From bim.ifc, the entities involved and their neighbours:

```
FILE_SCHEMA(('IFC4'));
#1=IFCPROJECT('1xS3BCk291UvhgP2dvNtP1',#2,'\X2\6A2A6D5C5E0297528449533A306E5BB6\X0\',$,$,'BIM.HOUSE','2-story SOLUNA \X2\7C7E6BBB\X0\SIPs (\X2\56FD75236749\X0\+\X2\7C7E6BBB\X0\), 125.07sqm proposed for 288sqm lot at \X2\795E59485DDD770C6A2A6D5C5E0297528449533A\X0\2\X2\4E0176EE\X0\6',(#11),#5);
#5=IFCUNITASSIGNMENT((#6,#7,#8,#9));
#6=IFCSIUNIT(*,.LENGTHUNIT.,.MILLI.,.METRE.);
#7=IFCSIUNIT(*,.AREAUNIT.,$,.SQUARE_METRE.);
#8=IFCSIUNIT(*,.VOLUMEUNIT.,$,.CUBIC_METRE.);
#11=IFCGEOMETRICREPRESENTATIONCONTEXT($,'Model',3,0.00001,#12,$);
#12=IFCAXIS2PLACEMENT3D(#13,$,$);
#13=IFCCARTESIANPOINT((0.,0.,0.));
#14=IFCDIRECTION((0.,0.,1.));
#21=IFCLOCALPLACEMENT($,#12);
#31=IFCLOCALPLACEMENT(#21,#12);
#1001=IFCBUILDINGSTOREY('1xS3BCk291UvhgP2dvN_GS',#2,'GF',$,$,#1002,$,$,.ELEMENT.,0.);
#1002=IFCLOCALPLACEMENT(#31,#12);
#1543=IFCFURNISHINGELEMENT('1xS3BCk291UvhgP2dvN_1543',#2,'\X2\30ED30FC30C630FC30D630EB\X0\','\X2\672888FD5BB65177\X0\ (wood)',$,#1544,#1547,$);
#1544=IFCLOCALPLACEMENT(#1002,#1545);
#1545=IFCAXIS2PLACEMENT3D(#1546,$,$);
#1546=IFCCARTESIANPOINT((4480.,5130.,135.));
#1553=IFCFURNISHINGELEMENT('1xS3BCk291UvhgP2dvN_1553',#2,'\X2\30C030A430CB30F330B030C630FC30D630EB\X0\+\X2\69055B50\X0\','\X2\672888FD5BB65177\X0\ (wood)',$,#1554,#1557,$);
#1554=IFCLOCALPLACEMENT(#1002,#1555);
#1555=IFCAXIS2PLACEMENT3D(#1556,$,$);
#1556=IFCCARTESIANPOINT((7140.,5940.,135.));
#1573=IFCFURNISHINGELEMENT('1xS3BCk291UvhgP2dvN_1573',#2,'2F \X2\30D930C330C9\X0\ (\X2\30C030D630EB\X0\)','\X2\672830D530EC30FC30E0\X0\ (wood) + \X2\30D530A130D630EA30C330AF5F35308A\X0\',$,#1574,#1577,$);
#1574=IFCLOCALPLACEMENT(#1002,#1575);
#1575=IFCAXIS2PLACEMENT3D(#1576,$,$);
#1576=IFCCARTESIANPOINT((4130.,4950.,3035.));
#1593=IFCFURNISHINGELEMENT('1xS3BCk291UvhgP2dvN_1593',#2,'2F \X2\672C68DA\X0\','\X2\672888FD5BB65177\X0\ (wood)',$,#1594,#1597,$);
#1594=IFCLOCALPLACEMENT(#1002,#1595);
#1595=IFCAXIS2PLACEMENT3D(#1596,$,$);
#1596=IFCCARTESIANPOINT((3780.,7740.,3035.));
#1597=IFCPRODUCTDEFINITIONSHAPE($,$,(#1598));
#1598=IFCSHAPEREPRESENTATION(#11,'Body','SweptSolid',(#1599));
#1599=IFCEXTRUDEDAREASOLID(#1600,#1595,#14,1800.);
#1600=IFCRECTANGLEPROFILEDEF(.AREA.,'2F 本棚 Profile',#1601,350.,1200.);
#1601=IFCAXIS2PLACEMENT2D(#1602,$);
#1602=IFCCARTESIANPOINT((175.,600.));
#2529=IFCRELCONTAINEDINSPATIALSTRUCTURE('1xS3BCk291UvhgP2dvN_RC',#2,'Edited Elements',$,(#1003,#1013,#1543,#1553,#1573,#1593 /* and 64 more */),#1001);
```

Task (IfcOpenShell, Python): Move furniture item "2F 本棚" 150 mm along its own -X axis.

```python
import ifcopenshell
import ifcopenshell.api.geometry
import ifcopenshell.util.placement
import ifcopenshell.util.unit

model = ifcopenshell.open("bim.ifc")
unit_scale = ifcopenshell.util.unit.calculate_unit_scale(model)

item = model.by_id(1593)
matrix = ifcopenshell.util.placement.get_local_placement(item.ObjectPlacement)
matrix[:3, 3] -= matrix[:3, 0] * 0.15 / unit_scale
ifcopenshell.api.geometry.edit_object_placement(model, product=item, matrix=matrix, is_si=False)

print(ifcopenshell.util.placement.get_local_placement(item.ObjectPlacement).round(3) + 0.0)

model.write("bim-out.ifc")
```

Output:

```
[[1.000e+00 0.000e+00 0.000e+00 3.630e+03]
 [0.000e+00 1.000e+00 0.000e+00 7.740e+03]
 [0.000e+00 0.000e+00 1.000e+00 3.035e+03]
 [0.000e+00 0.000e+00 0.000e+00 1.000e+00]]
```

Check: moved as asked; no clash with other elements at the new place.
